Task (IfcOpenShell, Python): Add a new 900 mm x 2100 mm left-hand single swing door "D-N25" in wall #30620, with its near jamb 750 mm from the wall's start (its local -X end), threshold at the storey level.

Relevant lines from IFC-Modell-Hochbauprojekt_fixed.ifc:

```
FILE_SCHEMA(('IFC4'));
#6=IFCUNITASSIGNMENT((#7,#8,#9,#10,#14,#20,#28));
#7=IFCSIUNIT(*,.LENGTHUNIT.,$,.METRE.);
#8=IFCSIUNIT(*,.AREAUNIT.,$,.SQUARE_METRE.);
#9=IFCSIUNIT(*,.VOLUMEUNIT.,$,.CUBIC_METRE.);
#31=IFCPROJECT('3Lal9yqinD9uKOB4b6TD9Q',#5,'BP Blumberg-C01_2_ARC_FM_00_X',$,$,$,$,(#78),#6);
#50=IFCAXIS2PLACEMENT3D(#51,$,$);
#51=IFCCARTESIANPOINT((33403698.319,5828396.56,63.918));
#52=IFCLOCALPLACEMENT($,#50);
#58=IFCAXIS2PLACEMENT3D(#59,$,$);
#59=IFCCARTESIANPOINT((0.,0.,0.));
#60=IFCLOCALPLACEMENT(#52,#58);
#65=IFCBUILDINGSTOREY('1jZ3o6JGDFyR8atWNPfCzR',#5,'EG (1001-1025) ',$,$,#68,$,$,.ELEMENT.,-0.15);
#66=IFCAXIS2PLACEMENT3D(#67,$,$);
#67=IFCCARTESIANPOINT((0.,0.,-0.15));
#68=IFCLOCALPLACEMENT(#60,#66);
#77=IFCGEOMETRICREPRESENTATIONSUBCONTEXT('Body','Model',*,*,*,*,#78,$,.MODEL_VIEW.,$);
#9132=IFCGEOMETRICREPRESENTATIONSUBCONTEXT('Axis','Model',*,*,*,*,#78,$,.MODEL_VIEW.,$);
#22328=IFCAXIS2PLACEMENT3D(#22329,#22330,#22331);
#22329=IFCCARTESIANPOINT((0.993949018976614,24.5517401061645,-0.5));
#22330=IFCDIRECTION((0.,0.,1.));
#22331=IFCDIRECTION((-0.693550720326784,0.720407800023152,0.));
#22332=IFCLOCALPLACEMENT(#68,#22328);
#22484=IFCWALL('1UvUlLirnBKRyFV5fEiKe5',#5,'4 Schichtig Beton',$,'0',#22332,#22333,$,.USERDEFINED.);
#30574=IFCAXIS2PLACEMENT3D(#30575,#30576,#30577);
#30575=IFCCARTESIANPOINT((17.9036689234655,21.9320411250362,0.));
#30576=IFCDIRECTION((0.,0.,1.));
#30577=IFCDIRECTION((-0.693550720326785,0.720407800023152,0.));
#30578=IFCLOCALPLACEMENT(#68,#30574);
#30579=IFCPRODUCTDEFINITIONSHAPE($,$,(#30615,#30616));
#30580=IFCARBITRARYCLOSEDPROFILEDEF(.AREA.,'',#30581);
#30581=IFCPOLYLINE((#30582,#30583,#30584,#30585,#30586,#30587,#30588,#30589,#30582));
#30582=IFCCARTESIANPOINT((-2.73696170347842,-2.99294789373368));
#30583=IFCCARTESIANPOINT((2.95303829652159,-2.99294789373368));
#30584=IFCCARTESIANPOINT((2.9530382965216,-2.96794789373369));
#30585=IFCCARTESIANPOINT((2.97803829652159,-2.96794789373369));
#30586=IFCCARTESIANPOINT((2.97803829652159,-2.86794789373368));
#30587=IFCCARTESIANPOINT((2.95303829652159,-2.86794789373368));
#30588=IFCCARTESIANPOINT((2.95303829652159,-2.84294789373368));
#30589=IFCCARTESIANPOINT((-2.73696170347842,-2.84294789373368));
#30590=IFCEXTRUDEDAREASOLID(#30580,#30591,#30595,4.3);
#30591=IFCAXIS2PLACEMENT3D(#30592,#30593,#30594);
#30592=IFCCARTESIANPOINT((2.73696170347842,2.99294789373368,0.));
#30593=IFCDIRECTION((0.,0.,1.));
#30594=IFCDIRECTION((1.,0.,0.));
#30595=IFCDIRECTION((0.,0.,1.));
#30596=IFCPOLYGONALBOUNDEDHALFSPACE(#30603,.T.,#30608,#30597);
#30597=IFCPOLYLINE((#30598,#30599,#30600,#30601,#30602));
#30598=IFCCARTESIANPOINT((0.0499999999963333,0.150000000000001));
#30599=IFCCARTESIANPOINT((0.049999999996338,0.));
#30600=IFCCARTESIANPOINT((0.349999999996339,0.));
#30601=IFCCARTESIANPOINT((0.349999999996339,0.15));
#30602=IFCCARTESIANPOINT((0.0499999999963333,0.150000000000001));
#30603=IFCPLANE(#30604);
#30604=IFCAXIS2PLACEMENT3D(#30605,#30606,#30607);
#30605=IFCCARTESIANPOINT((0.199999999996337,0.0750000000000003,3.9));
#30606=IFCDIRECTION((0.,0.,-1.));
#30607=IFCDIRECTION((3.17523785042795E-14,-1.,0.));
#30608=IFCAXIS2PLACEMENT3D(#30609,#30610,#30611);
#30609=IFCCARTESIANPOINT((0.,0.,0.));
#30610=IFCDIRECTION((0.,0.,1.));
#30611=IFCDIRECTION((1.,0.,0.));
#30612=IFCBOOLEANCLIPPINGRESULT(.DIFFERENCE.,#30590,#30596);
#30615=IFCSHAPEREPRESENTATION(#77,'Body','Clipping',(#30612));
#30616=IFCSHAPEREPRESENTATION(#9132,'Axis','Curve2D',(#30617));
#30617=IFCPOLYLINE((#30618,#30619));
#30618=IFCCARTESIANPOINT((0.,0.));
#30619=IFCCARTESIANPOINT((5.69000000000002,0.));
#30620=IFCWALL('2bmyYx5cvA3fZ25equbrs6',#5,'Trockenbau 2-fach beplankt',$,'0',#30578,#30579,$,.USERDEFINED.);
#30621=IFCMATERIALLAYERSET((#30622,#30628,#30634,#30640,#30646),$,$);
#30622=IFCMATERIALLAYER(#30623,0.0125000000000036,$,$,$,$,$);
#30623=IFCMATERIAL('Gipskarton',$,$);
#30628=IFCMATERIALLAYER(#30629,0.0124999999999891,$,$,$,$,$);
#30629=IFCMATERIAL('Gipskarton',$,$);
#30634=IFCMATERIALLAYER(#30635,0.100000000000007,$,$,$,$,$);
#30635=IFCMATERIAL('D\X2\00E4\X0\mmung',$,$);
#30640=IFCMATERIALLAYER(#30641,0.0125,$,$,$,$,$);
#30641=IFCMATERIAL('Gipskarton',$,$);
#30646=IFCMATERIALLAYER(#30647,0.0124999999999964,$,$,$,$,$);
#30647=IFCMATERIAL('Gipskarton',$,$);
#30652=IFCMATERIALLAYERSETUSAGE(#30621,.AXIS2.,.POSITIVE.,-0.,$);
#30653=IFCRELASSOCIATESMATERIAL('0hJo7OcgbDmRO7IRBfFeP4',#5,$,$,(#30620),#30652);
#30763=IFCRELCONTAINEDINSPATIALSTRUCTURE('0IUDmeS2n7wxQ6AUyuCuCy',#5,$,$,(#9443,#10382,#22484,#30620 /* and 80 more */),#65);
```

```python
import numpy as np
import ifcopenshell
import ifcopenshell.api.feature
import ifcopenshell.api.geometry
import ifcopenshell.api.root
import ifcopenshell.api.spatial
import ifcopenshell.geom
import ifcopenshell.util.element
import ifcopenshell.util.placement
import ifcopenshell.util.representation
import ifcopenshell.util.shape
import ifcopenshell.util.unit

model = ifcopenshell.open("IFC-Modell-Hochbauprojekt_fixed.ifc")
unit_scale = ifcopenshell.util.unit.calculate_unit_scale(model)
settings = ifcopenshell.geom.settings()


def volume(element):
    """Net volume in cubic metres, openings subtracted."""
    shape = ifcopenshell.geom.create_shape(settings, element)
    return ifcopenshell.util.shape.get_volume(shape.geometry)


wall = model.by_guid("2bmyYx5cvA3fZ25equbrs6")
storey = ifcopenshell.util.element.get_container(wall, ifc_class="IfcBuildingStorey")
context = ifcopenshell.util.representation.get_context(model, "Model", "Body", "MODEL_VIEW")
before = volume(wall)

width, height, from_end, sill = 0.9, 2.1, 0.75, 0.0  # metres

# The wall runs along its own X axis, and the end named is its -X end.
wall_shape = ifcopenshell.geom.create_shape(settings, wall)
x, y, z = ifcopenshell.util.shape.get_vertices(wall_shape.geometry).T
start = x.min() + from_end
face, thickness = float(y.min()), float(y.max() - y.min())
wall_matrix = ifcopenshell.util.placement.get_local_placement(wall.ObjectPlacement)
level = ifcopenshell.util.placement.get_local_placement(storey.ObjectPlacement)[2, 3]


def in_wall(x, y):
    """Placement at x, y metres in the wall's axes, at sill height."""
    matrix = wall_matrix.copy()
    matrix[:, 3] = wall_matrix @ np.array([x / unit_scale, y / unit_scale, 0.0, 1.0])
    matrix[2, 3] = level + sill / unit_scale
    return matrix


# Opening: a box that overshoots both wall faces by 50 mm.
opening = ifcopenshell.api.root.create_entity(model, ifc_class="IfcOpeningElement", predefined_type="OPENING")
box = ifcopenshell.api.geometry.add_wall_representation(
    model, context=context, length=width, height=height, thickness=thickness + 0.1
)
ifcopenshell.api.geometry.assign_representation(model, product=opening, representation=box)
ifcopenshell.api.geometry.edit_object_placement(model, product=opening, matrix=in_wall(start, face - 0.05), is_si=False)
ifcopenshell.api.feature.add_feature(model, feature=opening, element=wall)

door = ifcopenshell.api.root.create_entity(model, ifc_class="IfcDoor", name="D-N25", predefined_type="DOOR")
door.OverallWidth, door.OverallHeight = width / unit_scale, height / unit_scale
door.OperationType = "SINGLE_SWING_LEFT"
body = ifcopenshell.api.geometry.add_door_representation(
    model,
    context=context,
    overall_width=door.OverallWidth,
    overall_height=door.OverallHeight,
    operation_type="SINGLE_SWING_LEFT",
    lining_properties={"LiningDepth": thickness / unit_scale, "ThresholdDepth": thickness / unit_scale},
)
ifcopenshell.api.geometry.assign_representation(model, product=door, representation=body)
ifcopenshell.api.spatial.assign_container(model, products=[door], relating_structure=storey)
ifcopenshell.api.feature.add_filling(model, opening=opening, element=door)

# The lining spans the wall, so the door starts at the wall face.
ifcopenshell.api.geometry.edit_object_placement(model, product=door, matrix=in_wall(start, face), is_si=False)

after = volume(wall)

print(f"wall volume {before:.3f} -> {after:.3f} m3")

model.write("IFC-Modell-Hochbauprojekt_fixed_edited.ifc")
```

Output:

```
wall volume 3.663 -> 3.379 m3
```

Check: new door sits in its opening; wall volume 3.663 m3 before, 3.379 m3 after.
